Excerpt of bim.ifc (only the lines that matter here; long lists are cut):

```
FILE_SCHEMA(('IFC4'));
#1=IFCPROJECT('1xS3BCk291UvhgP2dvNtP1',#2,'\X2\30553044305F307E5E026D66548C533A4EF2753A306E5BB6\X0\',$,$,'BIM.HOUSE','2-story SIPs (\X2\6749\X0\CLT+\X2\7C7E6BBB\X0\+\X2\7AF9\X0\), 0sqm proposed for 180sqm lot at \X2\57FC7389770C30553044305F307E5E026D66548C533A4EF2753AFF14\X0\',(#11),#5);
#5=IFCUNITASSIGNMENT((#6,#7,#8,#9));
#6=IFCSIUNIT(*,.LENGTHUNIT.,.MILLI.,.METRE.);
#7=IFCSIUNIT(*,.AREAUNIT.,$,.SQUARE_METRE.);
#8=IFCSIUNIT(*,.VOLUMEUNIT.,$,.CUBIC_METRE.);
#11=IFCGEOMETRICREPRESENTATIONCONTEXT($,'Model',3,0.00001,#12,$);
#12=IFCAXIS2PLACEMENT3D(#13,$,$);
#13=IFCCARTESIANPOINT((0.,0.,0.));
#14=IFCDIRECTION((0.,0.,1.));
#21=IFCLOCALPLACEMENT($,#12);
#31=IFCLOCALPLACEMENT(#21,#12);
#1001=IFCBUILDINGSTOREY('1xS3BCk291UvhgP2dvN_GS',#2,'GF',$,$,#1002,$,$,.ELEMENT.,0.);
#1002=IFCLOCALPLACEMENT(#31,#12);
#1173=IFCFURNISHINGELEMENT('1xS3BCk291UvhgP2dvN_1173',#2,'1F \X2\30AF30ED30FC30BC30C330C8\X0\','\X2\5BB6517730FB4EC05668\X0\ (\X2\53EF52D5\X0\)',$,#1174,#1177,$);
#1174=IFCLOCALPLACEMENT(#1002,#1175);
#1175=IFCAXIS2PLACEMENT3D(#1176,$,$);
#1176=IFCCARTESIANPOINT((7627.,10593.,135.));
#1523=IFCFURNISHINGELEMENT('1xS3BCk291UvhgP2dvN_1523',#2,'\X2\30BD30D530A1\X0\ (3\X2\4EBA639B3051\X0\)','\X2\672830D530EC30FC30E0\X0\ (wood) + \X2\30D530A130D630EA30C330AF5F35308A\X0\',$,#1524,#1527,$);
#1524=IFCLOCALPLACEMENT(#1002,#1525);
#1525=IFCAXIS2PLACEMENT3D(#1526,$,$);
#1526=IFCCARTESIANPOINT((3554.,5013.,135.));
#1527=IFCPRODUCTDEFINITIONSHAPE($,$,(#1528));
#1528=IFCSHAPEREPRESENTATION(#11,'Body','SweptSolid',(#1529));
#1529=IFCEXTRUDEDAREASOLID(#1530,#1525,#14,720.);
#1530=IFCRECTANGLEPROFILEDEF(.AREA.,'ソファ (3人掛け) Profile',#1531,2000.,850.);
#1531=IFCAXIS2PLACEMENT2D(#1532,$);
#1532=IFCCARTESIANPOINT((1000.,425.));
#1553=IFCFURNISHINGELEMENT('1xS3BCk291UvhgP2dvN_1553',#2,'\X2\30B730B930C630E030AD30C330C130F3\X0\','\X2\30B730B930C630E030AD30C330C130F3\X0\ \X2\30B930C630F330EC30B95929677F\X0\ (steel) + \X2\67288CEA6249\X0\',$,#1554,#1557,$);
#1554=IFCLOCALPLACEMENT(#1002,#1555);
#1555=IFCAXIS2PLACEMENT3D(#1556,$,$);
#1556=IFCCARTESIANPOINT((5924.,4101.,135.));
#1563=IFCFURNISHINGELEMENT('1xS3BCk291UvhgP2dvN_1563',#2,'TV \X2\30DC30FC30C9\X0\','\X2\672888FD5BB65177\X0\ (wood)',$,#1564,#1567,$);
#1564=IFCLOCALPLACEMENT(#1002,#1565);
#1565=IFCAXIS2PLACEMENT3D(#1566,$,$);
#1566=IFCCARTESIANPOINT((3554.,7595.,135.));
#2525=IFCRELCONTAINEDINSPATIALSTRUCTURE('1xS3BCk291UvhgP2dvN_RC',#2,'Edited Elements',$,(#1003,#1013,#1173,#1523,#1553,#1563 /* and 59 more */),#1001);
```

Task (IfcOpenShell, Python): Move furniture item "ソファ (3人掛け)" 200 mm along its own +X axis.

```python
import ifcopenshell
import ifcopenshell.api.geometry
import ifcopenshell.util.placement

model = ifcopenshell.open("bim.ifc")

item = model.by_id(1523)
matrix = ifcopenshell.util.placement.get_local_placement(item.ObjectPlacement)
matrix[:3, 3] += matrix[:3, 0] * 200.0
ifcopenshell.api.geometry.edit_object_placement(model, product=item, matrix=matrix, is_si=False)

print(ifcopenshell.util.placement.get_local_placement(item.ObjectPlacement).round(3) + 0.0)

model.write("bim_updated.ifc")
```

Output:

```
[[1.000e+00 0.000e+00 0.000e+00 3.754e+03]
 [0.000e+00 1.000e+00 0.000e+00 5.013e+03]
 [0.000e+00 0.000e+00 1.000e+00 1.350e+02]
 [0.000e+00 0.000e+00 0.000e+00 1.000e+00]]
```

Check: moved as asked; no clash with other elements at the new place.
